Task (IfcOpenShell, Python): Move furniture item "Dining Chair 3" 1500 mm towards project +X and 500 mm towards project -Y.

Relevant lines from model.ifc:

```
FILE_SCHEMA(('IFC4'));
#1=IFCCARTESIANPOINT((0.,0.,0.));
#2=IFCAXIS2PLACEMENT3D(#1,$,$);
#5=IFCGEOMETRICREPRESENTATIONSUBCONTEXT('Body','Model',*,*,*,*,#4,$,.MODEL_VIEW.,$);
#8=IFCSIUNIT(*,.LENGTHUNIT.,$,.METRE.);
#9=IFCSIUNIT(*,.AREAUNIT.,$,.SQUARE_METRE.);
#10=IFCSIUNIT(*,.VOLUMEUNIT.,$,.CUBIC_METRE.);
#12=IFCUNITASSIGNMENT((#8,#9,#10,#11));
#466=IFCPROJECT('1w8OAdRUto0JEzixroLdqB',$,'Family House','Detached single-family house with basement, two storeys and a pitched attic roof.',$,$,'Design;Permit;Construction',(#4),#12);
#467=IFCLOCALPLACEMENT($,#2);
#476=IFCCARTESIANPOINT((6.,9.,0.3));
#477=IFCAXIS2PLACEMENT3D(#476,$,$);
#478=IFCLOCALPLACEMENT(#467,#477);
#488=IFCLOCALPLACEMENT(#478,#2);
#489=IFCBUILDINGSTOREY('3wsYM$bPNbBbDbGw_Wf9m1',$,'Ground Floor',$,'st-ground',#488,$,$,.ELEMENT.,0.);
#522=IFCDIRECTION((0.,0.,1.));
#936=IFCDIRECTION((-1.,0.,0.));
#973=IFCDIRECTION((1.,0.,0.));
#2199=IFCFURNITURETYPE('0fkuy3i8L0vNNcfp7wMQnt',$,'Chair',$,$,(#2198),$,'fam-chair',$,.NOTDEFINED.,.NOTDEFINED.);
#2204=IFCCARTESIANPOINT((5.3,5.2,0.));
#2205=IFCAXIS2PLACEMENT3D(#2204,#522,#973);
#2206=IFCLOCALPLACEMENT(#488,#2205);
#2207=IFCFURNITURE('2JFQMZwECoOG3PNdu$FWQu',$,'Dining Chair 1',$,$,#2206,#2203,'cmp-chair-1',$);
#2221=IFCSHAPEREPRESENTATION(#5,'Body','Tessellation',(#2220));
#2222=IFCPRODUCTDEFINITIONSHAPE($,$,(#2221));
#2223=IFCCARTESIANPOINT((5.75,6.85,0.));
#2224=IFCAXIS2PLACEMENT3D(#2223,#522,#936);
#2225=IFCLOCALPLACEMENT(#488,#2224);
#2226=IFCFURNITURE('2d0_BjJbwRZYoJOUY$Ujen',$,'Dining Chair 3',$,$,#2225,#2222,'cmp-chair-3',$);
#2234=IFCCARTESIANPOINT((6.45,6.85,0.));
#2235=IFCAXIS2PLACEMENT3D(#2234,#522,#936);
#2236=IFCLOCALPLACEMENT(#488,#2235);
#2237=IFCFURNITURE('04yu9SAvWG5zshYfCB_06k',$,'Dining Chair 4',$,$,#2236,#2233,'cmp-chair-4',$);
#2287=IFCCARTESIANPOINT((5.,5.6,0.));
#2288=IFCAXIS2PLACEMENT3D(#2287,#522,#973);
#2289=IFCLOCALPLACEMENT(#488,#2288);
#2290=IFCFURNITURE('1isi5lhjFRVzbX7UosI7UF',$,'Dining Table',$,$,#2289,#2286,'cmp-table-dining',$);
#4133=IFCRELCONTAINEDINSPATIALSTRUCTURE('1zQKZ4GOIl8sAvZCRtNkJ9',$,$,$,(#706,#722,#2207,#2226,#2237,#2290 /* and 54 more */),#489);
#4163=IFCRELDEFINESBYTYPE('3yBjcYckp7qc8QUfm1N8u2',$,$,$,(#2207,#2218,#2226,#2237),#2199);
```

```python
import ifcopenshell
import ifcopenshell.api.geometry
import ifcopenshell.util.placement
import ifcopenshell.util.unit

model = ifcopenshell.open("model.ifc")
unit_scale = ifcopenshell.util.unit.calculate_unit_scale(model)

item = model.by_guid("2d0_BjJbwRZYoJOUY$Ujen")
matrix = ifcopenshell.util.placement.get_local_placement(item.ObjectPlacement)
matrix[0, 3] += 1.5 / unit_scale
matrix[1, 3] -= 0.5 / unit_scale
ifcopenshell.api.geometry.edit_object_placement(model, product=item, matrix=matrix, is_si=False)

print(ifcopenshell.util.placement.get_local_placement(item.ObjectPlacement).round(3) + 0.0)

model.write("model_edited.ifc")
```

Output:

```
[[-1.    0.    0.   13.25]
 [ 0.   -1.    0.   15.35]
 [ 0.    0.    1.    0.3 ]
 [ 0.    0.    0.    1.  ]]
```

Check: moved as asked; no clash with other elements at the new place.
